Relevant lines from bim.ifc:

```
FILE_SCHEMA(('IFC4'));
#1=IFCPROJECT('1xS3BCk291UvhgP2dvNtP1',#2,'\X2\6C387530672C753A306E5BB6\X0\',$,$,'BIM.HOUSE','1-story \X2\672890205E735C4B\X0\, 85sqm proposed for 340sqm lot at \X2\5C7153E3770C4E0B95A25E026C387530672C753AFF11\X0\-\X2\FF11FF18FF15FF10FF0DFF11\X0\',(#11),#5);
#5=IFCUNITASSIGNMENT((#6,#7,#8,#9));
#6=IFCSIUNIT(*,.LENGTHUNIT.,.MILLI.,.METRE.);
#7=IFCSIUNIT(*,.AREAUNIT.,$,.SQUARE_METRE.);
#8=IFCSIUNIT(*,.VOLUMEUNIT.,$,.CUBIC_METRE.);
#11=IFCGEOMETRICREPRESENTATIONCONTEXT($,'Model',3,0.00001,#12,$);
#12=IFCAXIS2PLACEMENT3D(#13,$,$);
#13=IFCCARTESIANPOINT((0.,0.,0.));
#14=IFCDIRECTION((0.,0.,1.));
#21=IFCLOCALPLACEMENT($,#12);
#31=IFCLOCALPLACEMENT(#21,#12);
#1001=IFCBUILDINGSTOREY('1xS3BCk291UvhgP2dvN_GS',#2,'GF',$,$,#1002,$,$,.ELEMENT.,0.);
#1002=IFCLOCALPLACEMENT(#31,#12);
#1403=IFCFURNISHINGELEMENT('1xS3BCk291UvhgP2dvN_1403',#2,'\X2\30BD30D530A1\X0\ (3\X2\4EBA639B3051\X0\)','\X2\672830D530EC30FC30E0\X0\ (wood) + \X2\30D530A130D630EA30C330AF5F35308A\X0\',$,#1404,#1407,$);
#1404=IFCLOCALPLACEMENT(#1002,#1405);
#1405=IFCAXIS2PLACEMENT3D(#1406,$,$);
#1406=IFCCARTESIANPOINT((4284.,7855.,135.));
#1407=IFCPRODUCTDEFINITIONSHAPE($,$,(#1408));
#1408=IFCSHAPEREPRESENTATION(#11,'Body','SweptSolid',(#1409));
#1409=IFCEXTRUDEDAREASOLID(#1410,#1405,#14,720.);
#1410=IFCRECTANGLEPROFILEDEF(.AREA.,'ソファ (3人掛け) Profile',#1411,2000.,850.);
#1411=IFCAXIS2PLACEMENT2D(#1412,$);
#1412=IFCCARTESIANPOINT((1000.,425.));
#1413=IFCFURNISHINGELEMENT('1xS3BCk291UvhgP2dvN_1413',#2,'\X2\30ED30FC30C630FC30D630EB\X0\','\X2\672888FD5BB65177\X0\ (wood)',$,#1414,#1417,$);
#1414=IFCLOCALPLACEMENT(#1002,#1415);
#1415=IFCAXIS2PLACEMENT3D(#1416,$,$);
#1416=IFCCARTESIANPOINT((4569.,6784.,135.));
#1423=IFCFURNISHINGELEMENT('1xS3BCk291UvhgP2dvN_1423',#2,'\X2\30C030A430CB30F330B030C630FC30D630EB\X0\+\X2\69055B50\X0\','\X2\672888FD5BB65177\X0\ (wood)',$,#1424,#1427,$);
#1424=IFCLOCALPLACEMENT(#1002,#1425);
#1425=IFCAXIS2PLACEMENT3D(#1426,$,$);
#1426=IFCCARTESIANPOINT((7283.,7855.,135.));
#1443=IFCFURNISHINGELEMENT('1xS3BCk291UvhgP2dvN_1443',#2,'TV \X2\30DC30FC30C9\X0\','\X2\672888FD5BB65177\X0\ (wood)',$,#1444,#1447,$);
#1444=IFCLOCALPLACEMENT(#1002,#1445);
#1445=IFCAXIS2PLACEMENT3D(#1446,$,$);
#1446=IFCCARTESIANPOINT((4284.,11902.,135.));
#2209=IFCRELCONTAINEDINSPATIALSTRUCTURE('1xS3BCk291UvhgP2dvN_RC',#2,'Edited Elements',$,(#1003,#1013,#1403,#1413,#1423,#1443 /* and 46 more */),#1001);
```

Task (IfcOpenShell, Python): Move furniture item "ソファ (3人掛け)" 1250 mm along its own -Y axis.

```python
import ifcopenshell
import ifcopenshell.api.geometry
import ifcopenshell.util.placement
import ifcopenshell.util.unit

model = ifcopenshell.open("bim.ifc")
unit_scale = ifcopenshell.util.unit.calculate_unit_scale(model)

item = model.by_guid("1xS3BCk291UvhgP2dvN_1403")
matrix = ifcopenshell.util.placement.get_local_placement(item.ObjectPlacement)
matrix[:3, 3] -= matrix[:3, 1] * 1.25 / unit_scale
ifcopenshell.api.geometry.edit_object_placement(model, product=item, matrix=matrix, is_si=False)

print(ifcopenshell.util.placement.get_local_placement(item.ObjectPlacement).round(3) + 0.0)

model.write("bim_rev.ifc")
```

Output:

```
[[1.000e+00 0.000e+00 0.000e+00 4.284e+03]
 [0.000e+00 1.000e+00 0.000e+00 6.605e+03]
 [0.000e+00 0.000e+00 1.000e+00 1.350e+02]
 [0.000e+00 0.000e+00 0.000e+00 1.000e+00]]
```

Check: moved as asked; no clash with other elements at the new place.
